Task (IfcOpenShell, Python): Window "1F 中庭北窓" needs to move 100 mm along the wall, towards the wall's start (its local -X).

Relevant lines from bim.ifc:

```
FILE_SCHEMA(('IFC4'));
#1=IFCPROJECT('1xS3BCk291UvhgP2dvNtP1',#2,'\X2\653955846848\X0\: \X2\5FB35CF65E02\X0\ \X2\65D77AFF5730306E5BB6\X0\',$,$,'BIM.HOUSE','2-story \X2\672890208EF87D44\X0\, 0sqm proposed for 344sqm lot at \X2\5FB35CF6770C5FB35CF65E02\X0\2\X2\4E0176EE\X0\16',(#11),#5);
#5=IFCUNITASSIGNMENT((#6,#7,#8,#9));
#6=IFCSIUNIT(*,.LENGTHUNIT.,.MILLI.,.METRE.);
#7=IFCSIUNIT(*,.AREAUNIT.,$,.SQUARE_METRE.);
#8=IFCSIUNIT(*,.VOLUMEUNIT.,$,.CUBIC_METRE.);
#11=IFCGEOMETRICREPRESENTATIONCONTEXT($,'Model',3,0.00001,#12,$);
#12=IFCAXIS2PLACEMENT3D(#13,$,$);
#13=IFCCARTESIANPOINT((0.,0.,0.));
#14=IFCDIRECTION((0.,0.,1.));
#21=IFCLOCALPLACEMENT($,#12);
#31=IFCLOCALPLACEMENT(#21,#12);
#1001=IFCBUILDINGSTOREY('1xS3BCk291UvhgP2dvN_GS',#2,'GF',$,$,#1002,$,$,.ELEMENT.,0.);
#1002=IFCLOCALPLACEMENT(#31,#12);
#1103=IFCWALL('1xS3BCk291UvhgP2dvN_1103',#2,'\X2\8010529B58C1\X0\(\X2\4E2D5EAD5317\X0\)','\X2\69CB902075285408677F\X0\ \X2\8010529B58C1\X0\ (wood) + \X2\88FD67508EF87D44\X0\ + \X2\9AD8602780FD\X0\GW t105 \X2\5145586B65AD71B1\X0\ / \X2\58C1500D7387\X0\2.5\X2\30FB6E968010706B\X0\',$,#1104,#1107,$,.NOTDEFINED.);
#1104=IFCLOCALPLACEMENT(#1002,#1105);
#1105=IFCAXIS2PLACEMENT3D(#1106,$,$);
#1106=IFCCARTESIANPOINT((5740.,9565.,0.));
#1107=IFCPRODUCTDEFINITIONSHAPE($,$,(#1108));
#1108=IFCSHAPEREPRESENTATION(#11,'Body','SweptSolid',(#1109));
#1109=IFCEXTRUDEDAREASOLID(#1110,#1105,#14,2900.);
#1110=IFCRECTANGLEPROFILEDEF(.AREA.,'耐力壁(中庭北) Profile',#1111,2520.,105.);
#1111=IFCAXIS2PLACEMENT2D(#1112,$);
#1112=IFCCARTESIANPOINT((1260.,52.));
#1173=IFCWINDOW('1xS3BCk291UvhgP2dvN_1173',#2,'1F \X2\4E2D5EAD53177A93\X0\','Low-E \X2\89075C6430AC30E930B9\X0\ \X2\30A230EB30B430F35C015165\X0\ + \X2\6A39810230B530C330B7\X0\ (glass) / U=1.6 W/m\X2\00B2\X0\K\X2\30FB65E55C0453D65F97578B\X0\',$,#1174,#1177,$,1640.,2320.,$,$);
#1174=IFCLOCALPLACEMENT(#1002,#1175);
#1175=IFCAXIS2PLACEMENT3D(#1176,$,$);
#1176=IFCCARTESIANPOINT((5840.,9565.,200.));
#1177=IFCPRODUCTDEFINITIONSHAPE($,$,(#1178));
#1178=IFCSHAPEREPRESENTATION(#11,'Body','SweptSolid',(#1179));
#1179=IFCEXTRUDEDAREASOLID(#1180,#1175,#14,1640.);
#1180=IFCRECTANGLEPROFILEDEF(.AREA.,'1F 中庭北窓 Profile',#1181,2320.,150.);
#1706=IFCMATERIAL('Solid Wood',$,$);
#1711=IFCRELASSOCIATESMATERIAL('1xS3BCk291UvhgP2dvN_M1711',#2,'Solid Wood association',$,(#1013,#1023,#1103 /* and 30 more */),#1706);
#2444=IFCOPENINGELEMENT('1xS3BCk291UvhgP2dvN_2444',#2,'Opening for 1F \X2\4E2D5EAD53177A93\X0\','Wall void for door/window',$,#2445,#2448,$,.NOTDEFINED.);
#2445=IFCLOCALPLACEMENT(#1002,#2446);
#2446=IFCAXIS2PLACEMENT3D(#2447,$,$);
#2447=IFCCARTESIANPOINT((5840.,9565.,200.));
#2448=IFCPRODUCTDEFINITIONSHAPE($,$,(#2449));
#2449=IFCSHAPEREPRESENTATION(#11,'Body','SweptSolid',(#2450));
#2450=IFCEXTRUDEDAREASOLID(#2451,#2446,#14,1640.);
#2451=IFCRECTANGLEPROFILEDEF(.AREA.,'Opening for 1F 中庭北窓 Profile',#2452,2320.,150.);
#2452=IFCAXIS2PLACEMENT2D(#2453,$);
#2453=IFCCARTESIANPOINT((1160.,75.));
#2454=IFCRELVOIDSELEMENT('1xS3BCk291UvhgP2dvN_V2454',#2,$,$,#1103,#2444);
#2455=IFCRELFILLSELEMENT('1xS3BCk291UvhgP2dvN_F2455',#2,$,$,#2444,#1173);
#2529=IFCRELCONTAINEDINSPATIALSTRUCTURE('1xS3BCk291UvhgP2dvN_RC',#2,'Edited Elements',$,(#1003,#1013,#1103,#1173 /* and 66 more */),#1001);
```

```python
import ifcopenshell
import ifcopenshell.api.geometry
import ifcopenshell.util.placement

model = ifcopenshell.open("bim.ifc")

window = model.by_guid("1xS3BCk291UvhgP2dvN_1173")
opening = window.FillsVoids[0].RelatingOpeningElement
wall = opening.VoidsElements[0].RelatingBuildingElement

wall_matrix = ifcopenshell.util.placement.get_local_placement(wall.ObjectPlacement)
shift = wall_matrix[:3, 0] * -100.0
before = ifcopenshell.util.placement.get_local_placement(window.ObjectPlacement)[:3, 3].copy()

# The window is not placed relative to its opening, so move both.
for product in (opening, window):
    matrix = ifcopenshell.util.placement.get_local_placement(product.ObjectPlacement)
    matrix[:3, 3] += shift
    ifcopenshell.api.geometry.edit_object_placement(model, product=product, matrix=matrix, is_si=False)

after = ifcopenshell.util.placement.get_local_placement(window.ObjectPlacement)[:3, 3]
print("window moved by", (after - before).round(3) + 0.0)

model.write("bim_rev.ifc")
```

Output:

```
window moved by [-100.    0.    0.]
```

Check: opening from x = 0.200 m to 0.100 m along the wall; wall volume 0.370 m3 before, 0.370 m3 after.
